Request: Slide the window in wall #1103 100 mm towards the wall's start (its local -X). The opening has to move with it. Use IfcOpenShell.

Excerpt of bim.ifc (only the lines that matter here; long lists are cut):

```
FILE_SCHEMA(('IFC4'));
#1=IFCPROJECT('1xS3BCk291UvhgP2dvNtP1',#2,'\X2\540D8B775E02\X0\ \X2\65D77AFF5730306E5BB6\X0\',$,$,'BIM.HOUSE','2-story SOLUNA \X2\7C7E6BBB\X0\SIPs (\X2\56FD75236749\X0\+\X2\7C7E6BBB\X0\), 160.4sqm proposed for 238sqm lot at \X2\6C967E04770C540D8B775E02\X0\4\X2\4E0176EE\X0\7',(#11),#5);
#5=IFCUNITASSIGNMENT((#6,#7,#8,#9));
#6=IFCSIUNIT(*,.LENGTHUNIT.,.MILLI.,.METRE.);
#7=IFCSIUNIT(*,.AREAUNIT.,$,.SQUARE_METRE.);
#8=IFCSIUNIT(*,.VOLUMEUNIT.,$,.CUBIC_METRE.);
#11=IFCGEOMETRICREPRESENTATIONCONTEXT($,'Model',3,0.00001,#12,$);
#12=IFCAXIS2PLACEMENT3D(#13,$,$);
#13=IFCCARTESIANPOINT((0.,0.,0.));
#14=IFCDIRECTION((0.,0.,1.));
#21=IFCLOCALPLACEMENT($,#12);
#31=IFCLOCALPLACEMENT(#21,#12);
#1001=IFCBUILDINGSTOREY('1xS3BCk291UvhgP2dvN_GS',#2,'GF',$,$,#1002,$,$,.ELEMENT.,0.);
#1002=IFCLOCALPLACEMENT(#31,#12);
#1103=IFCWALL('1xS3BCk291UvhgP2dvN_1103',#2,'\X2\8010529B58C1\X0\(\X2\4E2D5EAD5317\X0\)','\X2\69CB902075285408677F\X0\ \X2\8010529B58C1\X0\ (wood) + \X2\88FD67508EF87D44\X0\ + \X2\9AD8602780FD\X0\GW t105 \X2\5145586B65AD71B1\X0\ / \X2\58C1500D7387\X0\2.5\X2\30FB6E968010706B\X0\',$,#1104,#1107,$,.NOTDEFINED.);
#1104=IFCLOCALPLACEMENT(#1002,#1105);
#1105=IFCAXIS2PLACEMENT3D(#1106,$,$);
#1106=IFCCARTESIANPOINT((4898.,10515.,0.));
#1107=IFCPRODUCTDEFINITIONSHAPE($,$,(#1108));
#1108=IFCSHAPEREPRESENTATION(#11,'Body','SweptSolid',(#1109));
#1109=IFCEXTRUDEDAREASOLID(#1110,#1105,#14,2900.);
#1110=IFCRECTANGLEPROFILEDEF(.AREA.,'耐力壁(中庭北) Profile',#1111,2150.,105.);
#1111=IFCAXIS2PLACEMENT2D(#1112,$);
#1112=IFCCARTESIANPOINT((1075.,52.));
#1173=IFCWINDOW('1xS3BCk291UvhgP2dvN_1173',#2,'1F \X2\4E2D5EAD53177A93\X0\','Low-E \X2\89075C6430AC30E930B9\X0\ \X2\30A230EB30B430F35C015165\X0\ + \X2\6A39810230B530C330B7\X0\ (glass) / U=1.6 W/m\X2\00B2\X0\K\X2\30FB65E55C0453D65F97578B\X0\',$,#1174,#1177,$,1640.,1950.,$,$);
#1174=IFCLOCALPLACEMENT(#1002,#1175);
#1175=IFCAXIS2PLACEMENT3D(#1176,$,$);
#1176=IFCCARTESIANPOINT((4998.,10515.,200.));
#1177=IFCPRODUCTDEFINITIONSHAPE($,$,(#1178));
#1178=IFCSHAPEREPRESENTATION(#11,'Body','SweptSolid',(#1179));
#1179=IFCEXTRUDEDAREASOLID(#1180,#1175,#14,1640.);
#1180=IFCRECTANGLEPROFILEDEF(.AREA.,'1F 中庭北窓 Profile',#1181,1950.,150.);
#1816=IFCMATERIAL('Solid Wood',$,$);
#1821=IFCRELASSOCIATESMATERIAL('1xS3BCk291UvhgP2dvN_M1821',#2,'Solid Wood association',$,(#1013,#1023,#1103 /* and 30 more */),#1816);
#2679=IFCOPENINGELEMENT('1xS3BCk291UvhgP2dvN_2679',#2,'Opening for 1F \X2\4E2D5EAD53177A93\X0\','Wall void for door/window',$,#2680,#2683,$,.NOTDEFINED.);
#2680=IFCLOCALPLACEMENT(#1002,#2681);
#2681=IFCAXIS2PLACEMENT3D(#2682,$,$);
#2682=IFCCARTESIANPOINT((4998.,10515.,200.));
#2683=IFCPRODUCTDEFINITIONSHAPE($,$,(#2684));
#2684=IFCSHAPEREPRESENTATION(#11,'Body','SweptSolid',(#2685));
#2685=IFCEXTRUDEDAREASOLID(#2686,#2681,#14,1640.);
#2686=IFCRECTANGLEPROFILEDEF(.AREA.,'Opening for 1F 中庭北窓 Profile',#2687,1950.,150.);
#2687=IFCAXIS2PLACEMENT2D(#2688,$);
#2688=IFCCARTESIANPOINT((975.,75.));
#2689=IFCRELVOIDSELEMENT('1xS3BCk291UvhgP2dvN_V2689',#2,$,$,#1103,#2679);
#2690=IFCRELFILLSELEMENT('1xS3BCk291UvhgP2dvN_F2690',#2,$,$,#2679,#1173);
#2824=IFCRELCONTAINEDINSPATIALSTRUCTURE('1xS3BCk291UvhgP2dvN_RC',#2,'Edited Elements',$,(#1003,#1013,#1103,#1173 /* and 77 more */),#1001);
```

```python
import ifcopenshell
import ifcopenshell.api.geometry
import ifcopenshell.util.placement

model = ifcopenshell.open("bim.ifc")

window = model.by_guid("1xS3BCk291UvhgP2dvN_1173")
opening = window.FillsVoids[0].RelatingOpeningElement
wall = opening.VoidsElements[0].RelatingBuildingElement

wall_matrix = ifcopenshell.util.placement.get_local_placement(wall.ObjectPlacement)
shift = wall_matrix[:3, 0] * -100.0
before = ifcopenshell.util.placement.get_local_placement(window.ObjectPlacement)[:3, 3].copy()

# The window is not placed relative to its opening, so move both.
for product in (opening, window):
    matrix = ifcopenshell.util.placement.get_local_placement(product.ObjectPlacement)
    matrix[:3, 3] += shift
    ifcopenshell.api.geometry.edit_object_placement(model, product=product, matrix=matrix, is_si=False)

after = ifcopenshell.util.placement.get_local_placement(window.ObjectPlacement)[:3, 3]
print("window moved by", (after - before).round(3) + 0.0)

model.write("bim-out.ifc")
```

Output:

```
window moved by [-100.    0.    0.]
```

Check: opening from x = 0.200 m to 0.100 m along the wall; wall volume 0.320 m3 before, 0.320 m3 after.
